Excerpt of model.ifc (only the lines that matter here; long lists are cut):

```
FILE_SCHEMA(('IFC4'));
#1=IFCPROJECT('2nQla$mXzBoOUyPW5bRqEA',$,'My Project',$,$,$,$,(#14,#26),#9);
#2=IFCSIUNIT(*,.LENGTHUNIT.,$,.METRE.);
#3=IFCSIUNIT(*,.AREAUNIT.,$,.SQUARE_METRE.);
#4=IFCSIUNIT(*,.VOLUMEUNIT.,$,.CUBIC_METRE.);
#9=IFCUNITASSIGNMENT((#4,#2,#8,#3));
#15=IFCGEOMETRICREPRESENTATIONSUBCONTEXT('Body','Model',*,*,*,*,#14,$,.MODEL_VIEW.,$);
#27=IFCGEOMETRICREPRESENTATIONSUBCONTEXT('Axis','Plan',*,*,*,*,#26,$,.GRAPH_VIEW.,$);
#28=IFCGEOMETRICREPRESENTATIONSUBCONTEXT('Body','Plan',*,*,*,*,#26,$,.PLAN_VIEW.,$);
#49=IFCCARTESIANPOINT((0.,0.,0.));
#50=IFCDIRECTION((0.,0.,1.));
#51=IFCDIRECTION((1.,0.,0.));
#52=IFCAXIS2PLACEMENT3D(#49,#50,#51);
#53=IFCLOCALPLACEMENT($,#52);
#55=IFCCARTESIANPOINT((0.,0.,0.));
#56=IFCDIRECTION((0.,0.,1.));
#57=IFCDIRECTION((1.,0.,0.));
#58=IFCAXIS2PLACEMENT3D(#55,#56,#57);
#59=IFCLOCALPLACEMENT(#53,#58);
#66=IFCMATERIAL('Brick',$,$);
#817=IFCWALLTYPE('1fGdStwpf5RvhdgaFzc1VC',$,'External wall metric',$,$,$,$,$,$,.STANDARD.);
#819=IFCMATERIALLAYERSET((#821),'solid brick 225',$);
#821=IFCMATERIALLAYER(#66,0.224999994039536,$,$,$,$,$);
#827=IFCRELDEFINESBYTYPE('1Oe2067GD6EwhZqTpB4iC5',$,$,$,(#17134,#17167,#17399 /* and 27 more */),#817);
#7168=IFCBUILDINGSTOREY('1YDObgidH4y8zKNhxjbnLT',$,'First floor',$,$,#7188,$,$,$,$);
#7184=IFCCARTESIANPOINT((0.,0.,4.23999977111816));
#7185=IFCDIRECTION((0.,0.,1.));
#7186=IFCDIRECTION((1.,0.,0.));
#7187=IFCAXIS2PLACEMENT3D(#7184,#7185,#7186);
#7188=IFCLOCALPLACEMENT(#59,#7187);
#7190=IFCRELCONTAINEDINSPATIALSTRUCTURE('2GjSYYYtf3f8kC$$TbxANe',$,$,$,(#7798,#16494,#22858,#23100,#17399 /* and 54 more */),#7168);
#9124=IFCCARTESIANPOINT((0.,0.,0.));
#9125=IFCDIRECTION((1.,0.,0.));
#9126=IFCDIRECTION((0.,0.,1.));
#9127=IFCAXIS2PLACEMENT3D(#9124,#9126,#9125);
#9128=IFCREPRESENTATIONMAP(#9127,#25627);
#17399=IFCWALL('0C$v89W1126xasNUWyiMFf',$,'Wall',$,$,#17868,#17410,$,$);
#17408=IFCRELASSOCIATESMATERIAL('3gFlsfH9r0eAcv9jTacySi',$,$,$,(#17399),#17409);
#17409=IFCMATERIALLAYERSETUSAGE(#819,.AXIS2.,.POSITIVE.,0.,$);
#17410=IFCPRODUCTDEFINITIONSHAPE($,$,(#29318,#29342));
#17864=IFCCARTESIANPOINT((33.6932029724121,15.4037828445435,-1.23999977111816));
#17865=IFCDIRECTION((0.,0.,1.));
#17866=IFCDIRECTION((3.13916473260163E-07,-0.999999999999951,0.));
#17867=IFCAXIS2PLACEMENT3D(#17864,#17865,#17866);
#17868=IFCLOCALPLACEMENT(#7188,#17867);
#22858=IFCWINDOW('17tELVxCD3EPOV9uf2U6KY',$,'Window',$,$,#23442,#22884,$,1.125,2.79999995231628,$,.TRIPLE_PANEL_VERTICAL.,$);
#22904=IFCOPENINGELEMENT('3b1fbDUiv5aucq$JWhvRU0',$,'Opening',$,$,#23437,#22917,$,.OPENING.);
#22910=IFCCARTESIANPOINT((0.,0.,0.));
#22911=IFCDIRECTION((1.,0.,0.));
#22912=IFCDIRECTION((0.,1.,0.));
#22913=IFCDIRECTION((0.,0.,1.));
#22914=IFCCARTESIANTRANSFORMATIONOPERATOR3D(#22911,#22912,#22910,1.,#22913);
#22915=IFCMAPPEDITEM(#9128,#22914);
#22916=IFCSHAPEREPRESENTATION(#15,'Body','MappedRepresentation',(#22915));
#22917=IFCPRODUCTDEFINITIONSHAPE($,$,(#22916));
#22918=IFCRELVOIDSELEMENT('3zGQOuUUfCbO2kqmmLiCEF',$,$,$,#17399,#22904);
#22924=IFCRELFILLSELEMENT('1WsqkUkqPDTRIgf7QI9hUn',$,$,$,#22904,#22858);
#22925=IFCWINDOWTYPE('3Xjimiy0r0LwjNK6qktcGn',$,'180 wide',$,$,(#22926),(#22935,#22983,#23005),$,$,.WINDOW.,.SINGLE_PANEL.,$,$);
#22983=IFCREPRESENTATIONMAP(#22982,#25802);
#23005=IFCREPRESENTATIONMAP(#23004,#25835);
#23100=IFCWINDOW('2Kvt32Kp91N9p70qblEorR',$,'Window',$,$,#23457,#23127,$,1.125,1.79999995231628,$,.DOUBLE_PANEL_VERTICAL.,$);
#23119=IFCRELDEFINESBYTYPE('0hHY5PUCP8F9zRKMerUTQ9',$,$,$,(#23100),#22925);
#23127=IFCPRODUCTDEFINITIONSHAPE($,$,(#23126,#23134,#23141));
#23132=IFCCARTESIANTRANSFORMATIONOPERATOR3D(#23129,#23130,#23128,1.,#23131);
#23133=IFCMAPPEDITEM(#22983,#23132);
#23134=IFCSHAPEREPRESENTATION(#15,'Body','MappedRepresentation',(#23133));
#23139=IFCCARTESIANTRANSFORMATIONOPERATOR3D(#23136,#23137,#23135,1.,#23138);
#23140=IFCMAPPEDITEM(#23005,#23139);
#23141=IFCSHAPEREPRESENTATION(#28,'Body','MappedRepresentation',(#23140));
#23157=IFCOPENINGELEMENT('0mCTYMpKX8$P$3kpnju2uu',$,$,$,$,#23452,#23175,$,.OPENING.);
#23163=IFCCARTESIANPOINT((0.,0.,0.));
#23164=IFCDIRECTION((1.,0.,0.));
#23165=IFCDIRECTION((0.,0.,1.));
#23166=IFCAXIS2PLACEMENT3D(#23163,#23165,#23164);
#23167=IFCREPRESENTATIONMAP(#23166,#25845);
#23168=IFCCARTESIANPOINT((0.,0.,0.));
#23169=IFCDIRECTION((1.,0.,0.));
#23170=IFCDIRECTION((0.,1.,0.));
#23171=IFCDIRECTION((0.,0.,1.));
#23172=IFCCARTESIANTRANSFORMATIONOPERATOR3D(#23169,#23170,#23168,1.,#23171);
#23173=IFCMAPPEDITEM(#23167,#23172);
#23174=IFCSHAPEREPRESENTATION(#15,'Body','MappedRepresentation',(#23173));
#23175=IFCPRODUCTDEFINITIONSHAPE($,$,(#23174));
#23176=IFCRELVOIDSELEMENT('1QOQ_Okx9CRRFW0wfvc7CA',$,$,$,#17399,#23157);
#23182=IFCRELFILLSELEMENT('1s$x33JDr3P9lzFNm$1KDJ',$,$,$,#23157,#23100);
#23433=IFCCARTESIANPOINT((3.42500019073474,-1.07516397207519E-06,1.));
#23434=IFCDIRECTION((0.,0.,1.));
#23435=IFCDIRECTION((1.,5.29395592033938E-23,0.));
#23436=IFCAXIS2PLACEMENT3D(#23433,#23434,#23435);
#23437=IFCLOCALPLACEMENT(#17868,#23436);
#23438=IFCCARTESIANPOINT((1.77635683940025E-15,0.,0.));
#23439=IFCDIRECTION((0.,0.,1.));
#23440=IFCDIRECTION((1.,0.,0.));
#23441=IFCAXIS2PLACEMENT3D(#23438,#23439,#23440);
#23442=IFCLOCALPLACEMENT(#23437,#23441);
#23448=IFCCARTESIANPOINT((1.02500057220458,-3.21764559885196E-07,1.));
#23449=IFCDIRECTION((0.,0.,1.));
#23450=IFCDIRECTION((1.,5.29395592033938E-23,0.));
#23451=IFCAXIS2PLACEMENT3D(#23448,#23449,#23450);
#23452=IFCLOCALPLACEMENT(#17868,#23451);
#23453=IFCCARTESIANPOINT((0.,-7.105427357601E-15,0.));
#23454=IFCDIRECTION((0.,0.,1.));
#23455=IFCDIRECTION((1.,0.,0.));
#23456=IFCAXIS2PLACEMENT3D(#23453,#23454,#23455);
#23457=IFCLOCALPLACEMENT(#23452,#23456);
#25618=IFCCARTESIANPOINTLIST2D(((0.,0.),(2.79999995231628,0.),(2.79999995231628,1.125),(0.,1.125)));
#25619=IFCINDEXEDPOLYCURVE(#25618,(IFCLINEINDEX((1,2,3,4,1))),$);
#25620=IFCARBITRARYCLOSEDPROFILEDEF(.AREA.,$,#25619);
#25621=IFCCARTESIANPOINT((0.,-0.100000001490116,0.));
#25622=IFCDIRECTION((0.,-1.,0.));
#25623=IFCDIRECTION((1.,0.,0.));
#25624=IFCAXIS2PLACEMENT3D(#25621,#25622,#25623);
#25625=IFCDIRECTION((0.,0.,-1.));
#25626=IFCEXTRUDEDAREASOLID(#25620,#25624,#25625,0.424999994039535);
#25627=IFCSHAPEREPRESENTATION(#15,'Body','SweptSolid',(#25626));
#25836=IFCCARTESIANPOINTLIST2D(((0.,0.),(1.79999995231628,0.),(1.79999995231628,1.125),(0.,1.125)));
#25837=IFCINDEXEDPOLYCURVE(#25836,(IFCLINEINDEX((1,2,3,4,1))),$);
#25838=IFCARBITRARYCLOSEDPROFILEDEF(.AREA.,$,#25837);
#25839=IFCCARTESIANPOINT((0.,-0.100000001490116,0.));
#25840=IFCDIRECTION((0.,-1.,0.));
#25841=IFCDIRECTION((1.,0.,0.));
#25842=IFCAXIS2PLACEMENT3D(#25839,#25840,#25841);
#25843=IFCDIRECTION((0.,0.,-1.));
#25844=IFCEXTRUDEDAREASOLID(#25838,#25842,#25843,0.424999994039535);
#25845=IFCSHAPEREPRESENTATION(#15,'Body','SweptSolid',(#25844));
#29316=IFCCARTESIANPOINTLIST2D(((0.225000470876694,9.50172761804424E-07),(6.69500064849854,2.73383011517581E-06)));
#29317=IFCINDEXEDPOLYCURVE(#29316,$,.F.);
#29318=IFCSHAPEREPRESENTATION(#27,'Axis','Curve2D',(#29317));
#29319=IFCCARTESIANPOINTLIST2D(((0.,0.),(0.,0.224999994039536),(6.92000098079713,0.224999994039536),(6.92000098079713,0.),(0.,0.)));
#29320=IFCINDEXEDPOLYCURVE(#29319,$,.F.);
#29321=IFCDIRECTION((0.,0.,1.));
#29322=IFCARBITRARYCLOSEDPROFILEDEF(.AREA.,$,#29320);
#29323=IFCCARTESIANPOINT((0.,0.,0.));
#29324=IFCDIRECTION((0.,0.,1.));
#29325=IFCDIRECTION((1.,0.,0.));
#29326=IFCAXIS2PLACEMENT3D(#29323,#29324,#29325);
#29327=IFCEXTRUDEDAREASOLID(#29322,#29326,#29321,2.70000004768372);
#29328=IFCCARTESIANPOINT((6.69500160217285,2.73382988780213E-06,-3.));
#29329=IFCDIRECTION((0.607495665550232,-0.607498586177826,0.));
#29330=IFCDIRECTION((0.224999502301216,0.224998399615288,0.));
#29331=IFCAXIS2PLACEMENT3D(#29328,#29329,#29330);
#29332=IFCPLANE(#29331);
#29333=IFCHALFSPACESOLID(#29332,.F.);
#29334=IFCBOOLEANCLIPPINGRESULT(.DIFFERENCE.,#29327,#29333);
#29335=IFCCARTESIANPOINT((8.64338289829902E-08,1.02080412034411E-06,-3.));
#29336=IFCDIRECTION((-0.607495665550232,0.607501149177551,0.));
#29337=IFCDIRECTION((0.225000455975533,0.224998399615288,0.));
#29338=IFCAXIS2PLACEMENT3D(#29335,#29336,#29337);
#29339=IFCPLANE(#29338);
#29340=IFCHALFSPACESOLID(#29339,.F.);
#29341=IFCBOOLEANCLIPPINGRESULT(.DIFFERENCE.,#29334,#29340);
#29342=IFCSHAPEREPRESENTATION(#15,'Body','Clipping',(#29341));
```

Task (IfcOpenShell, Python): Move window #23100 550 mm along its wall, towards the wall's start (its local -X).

```python
import ifcopenshell
import ifcopenshell.api.geometry
import ifcopenshell.util.placement
import ifcopenshell.util.unit

model = ifcopenshell.open("model.ifc")
unit_scale = ifcopenshell.util.unit.calculate_unit_scale(model)

window = model.by_id(23100)
opening = window.FillsVoids[0].RelatingOpeningElement
wall = opening.VoidsElements[0].RelatingBuildingElement

wall_matrix = ifcopenshell.util.placement.get_local_placement(wall.ObjectPlacement)
shift = wall_matrix[:3, 0] * -0.55 / unit_scale
before = ifcopenshell.util.placement.get_local_placement(window.ObjectPlacement)[:3, 3].copy()

# The window is placed relative to its opening, so it follows when the opening moves.
matrix = ifcopenshell.util.placement.get_local_placement(opening.ObjectPlacement)
matrix[:3, 3] += shift
ifcopenshell.api.geometry.edit_object_placement(
    model, product=opening, matrix=matrix, is_si=False, should_transform_children=True
)

after = ifcopenshell.util.placement.get_local_placement(window.ObjectPlacement)[:3, 3]
print("window moved by", (after - before).round(3) + 0.0)

model.write("model_updated.ifc")
```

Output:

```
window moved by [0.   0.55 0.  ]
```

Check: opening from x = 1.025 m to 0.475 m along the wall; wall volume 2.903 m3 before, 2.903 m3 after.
